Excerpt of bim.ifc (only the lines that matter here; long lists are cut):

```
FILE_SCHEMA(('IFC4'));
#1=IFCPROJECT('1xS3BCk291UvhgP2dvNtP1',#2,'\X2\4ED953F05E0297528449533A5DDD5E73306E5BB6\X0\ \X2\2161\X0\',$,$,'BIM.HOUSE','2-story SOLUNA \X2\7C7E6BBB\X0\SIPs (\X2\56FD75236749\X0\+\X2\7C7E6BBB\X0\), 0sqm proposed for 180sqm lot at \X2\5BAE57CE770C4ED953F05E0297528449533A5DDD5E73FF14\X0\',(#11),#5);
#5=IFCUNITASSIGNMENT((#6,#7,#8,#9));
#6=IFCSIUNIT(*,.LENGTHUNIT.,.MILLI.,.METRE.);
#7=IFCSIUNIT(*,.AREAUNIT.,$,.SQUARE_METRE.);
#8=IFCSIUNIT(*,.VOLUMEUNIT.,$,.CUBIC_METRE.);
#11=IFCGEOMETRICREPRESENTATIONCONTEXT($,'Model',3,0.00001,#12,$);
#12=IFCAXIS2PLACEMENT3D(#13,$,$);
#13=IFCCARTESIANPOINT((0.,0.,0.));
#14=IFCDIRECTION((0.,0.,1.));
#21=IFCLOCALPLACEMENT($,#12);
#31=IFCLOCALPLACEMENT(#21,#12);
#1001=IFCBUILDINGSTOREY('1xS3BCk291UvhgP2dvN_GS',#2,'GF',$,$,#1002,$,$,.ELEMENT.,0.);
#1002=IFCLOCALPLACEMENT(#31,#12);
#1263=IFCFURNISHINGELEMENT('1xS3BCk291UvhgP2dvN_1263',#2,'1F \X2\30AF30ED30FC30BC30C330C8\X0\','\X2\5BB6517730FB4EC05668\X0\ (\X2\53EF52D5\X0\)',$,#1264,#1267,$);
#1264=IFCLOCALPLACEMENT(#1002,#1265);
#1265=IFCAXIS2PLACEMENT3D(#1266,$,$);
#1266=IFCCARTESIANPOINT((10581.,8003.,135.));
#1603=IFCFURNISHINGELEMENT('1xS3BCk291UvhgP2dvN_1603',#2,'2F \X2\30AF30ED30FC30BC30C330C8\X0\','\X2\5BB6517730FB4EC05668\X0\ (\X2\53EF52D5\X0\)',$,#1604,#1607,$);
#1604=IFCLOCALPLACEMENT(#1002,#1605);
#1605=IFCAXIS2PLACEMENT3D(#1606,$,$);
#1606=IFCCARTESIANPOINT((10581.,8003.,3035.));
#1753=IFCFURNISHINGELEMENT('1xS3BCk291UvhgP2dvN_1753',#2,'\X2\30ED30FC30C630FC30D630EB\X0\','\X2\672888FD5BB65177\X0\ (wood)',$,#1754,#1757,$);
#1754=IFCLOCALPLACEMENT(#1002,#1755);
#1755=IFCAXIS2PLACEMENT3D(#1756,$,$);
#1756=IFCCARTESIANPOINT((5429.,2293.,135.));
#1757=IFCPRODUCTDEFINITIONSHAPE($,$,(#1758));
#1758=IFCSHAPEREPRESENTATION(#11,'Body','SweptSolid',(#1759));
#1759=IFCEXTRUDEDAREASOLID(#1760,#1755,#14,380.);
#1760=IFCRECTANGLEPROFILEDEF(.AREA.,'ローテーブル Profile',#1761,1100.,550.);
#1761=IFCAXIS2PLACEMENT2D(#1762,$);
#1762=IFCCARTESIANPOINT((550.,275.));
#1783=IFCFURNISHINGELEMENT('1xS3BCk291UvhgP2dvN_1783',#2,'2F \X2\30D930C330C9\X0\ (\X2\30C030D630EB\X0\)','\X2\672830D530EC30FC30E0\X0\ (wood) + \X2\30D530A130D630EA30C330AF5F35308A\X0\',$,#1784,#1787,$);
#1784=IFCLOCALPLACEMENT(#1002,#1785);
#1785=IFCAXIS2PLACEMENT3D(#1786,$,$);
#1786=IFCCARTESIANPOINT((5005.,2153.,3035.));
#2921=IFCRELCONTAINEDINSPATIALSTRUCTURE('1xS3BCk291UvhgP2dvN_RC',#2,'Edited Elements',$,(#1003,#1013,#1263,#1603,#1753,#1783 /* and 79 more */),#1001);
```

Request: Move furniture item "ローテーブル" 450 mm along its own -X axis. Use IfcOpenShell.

```python
import ifcopenshell
import ifcopenshell.api.geometry
import ifcopenshell.util.placement
import ifcopenshell.util.unit

model = ifcopenshell.open("bim.ifc")
unit_scale = ifcopenshell.util.unit.calculate_unit_scale(model)

item = model.by_guid("1xS3BCk291UvhgP2dvN_1753")
matrix = ifcopenshell.util.placement.get_local_placement(item.ObjectPlacement)
matrix[:3, 3] -= matrix[:3, 0] * 0.45 / unit_scale
ifcopenshell.api.geometry.edit_object_placement(model, product=item, matrix=matrix, is_si=False)

print(ifcopenshell.util.placement.get_local_placement(item.ObjectPlacement).round(3) + 0.0)

model.write("bim-out.ifc")
```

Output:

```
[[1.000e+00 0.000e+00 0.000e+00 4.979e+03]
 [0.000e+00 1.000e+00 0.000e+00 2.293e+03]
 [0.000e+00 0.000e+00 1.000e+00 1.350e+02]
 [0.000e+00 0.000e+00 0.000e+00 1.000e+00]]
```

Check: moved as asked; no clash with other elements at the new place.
